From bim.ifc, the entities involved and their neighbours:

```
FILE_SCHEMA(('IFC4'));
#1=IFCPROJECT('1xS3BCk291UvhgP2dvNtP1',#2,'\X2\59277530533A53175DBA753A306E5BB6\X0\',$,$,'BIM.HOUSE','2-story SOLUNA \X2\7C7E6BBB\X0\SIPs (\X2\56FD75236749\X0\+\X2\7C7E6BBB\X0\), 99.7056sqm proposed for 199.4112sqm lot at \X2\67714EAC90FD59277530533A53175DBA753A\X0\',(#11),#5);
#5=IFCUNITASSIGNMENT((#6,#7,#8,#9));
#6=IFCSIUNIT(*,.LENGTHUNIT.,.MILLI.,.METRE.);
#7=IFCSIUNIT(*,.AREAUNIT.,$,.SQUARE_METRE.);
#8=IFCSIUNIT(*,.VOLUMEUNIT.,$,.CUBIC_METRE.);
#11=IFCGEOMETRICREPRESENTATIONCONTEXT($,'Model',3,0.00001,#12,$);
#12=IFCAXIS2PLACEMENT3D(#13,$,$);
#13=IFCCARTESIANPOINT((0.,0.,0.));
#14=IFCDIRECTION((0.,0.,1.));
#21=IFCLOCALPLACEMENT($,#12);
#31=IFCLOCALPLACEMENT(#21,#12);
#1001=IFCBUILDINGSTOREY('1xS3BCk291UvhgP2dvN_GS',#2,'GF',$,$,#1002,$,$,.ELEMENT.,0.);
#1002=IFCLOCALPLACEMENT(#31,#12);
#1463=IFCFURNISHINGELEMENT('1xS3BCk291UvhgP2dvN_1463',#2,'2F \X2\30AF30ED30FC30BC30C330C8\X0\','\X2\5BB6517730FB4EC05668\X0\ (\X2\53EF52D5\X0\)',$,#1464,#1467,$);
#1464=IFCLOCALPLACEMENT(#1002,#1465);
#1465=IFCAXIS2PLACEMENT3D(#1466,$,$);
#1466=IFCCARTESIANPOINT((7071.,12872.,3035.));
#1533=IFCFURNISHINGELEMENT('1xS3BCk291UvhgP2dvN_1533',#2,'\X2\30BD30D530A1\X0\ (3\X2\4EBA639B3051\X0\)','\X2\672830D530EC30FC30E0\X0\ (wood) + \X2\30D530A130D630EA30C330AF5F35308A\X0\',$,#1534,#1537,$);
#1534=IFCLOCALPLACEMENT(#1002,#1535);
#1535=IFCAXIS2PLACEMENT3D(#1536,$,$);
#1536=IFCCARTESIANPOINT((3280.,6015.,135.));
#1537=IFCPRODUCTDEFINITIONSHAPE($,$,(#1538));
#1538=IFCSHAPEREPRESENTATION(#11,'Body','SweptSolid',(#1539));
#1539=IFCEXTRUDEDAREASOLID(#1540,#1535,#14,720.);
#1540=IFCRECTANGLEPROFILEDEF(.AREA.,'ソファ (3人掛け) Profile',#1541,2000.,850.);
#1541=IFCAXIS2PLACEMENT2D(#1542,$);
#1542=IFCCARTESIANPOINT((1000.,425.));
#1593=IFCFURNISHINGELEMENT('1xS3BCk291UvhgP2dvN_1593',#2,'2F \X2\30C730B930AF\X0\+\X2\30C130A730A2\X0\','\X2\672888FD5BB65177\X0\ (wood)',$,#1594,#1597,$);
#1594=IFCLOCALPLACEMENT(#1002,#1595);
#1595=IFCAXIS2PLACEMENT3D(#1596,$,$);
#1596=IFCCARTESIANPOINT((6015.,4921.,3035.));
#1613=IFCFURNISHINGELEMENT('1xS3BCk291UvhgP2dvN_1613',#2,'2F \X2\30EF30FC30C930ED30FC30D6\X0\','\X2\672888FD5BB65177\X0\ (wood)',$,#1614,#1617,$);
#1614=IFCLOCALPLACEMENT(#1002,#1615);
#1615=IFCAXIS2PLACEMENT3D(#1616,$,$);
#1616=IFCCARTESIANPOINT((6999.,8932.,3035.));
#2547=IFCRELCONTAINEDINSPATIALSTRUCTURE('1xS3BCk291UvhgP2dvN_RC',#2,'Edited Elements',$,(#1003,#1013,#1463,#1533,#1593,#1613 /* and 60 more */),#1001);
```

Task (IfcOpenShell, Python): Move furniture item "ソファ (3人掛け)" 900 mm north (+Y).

```python
import ifcopenshell
import ifcopenshell.api.geometry
import ifcopenshell.util.placement

model = ifcopenshell.open("bim.ifc")

item = model.by_id(1533)
matrix = ifcopenshell.util.placement.get_local_placement(item.ObjectPlacement)
matrix[1, 3] += 900.0
ifcopenshell.api.geometry.edit_object_placement(model, product=item, matrix=matrix, is_si=False)

print(ifcopenshell.util.placement.get_local_placement(item.ObjectPlacement).round(3) + 0.0)

model.write("bim_edited.ifc")
```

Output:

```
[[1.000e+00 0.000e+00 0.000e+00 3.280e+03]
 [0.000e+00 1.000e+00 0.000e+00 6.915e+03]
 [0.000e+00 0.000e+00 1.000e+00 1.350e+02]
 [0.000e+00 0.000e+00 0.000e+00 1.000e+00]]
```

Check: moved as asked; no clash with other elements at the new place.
